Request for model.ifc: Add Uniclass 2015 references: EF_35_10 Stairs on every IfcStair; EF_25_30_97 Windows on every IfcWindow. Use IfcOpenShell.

First a look at what the model holds.

```python
import ifcopenshell

model = ifcopenshell.open("model.ifc")
print(model.schema)
print("classifications:", [c.Name for c in model.by_type("IfcClassification")])
for ifc_class in ("IfcDoor", "IfcRoof", "IfcStair", "IfcWall", "IfcWindow"):
    print(ifc_class, len(model.by_type(ifc_class)))
```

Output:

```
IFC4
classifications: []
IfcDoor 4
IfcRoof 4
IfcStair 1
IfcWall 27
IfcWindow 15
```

```python
import ifcopenshell
import ifcopenshell.api.classification

model = ifcopenshell.open("model.ifc")

system = ifcopenshell.api.classification.add_classification(model, classification="Uniclass 2015")

codes = {
    "IfcStair": ("EF_35_10", "Stairs"),
    "IfcWindow": ("EF_25_30_97", "Windows"),
}
for ifc_class, (code, name) in codes.items():
    products = model.by_type(ifc_class)
    ifcopenshell.api.classification.add_reference(
        model, products=products, classification=system, identification=code, name=name
    )
    print(code, len(products))

model.write("model-out.ifc")
```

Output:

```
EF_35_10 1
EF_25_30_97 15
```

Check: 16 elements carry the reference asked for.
